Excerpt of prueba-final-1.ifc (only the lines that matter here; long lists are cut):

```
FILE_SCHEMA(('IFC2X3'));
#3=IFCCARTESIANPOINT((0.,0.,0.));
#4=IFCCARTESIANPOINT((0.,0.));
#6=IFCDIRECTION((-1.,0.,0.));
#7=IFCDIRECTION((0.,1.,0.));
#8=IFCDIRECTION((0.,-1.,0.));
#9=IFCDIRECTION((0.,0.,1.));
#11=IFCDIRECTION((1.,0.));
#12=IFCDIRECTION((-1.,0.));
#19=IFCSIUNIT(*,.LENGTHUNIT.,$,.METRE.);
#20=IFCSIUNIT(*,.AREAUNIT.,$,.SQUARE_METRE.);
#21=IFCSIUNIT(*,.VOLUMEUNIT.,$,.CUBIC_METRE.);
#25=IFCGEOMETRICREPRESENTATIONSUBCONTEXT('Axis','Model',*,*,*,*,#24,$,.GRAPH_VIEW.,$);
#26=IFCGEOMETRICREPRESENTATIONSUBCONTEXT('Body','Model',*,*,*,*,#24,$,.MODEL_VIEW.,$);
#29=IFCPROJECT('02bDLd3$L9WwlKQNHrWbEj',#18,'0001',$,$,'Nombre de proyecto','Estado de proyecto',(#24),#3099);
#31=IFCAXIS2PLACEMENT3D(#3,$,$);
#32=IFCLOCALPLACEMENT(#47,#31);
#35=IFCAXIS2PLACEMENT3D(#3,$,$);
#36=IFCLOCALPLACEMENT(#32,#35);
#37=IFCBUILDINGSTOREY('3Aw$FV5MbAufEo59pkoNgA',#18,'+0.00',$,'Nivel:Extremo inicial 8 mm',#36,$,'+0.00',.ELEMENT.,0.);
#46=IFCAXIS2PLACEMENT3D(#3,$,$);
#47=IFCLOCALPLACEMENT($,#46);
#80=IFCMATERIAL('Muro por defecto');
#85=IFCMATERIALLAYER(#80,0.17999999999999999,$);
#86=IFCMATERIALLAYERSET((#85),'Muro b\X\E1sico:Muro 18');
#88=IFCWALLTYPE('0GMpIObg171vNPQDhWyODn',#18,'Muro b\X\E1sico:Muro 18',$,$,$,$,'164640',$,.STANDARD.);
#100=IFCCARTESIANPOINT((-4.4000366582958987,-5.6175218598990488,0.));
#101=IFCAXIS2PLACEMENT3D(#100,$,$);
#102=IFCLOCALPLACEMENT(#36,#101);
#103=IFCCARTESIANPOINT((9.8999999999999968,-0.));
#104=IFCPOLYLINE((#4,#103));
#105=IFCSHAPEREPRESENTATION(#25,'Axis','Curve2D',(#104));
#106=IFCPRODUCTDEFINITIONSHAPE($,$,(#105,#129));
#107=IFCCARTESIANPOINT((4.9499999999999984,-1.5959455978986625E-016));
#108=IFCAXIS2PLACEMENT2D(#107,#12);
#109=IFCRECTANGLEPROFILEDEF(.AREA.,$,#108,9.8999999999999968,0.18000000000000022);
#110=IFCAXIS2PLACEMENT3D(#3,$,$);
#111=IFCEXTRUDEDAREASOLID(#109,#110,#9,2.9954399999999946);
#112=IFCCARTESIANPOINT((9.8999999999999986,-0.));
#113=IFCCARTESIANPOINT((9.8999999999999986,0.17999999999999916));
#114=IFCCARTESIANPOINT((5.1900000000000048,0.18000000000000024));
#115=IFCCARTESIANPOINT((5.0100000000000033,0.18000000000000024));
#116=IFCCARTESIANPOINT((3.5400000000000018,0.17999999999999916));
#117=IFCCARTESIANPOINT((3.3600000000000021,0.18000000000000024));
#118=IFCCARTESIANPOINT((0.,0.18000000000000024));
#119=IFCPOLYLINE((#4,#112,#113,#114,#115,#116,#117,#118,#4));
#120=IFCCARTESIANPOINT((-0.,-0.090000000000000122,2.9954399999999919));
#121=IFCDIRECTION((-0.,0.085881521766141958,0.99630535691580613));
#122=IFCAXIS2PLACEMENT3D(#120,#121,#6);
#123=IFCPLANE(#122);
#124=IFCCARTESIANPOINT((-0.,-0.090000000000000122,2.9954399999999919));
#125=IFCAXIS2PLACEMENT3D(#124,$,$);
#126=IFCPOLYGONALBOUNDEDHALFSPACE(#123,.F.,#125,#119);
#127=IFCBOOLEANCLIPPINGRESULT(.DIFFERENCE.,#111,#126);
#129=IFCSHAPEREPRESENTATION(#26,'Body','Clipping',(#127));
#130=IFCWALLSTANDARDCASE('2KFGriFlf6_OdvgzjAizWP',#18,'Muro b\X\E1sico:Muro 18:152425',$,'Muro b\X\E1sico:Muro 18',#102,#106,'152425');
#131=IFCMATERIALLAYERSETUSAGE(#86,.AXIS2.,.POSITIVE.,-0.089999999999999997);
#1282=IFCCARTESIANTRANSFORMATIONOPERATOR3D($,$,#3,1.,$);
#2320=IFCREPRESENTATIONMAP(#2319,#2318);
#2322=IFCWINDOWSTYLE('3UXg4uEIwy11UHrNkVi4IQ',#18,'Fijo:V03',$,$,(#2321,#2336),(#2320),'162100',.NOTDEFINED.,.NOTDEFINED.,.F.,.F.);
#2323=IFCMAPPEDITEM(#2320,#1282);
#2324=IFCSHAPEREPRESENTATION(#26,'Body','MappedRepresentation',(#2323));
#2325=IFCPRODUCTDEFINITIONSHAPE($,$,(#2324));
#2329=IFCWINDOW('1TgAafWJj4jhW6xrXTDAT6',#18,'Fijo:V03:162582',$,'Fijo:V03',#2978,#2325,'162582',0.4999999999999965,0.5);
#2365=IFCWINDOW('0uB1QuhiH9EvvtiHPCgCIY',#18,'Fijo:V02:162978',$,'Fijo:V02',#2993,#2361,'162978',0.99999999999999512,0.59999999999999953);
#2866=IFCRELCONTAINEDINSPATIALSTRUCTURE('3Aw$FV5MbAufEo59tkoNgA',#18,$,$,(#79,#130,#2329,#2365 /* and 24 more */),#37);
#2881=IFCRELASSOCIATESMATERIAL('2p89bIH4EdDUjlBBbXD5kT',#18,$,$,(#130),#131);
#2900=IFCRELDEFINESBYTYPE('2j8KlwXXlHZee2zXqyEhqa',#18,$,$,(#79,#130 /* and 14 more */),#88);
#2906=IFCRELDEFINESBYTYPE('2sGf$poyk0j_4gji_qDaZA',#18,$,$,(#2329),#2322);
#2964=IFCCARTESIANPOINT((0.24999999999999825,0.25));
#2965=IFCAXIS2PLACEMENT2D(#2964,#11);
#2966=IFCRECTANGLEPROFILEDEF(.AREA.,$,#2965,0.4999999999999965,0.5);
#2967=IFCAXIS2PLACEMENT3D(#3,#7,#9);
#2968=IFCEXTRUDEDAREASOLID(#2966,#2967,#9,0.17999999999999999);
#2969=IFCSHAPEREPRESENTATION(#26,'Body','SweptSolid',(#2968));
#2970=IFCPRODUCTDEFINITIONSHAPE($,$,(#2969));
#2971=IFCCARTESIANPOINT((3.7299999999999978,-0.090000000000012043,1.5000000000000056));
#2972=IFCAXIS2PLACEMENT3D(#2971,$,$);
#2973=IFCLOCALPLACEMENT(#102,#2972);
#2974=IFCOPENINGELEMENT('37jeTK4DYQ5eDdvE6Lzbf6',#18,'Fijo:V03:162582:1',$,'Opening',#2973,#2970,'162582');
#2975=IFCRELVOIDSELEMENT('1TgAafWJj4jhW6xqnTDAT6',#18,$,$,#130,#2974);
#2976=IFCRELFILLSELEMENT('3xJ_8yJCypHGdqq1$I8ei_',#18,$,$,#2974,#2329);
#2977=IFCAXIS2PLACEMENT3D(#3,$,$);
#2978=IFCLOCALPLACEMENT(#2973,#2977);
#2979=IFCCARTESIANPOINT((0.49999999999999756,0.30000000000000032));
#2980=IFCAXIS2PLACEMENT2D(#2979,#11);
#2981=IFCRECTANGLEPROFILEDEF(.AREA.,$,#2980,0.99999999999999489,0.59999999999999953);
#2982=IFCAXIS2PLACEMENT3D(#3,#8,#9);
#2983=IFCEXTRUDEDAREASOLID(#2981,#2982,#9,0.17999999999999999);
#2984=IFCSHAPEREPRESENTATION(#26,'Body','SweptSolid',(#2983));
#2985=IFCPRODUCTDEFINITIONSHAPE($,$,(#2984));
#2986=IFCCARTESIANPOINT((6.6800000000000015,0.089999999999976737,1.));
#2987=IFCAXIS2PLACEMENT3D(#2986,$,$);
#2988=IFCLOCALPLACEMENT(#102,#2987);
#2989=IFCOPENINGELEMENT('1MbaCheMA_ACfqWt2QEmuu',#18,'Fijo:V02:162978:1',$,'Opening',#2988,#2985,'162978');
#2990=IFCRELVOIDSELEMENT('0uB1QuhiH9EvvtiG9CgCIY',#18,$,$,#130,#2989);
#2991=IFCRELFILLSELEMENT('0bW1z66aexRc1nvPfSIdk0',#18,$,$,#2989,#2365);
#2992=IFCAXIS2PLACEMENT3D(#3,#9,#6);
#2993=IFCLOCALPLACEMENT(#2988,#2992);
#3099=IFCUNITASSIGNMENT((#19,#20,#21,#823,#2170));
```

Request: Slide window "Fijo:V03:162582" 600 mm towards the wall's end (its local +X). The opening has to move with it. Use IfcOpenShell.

```python
import ifcopenshell
import ifcopenshell.api.geometry
import ifcopenshell.util.placement

model = ifcopenshell.open("prueba-final-1.ifc")

window = model.by_guid("1TgAafWJj4jhW6xrXTDAT6")
opening = window.FillsVoids[0].RelatingOpeningElement
wall = opening.VoidsElements[0].RelatingBuildingElement

wall_matrix = ifcopenshell.util.placement.get_local_placement(wall.ObjectPlacement)
shift = wall_matrix[:3, 0] * 0.6
before = ifcopenshell.util.placement.get_local_placement(window.ObjectPlacement)[:3, 3].copy()

# The window is placed relative to its opening, so it follows when the opening moves.
matrix = ifcopenshell.util.placement.get_local_placement(opening.ObjectPlacement)
matrix[:3, 3] += shift
ifcopenshell.api.geometry.edit_object_placement(
    model, product=opening, matrix=matrix, is_si=False, should_transform_children=True
)

after = ifcopenshell.util.placement.get_local_placement(window.ObjectPlacement)[:3, 3]
print("window moved by", (after - before).round(3) + 0.0)

model.write("prueba-final-1_rev.ifc")
```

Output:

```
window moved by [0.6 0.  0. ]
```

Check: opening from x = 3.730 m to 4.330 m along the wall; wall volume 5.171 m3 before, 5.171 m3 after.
